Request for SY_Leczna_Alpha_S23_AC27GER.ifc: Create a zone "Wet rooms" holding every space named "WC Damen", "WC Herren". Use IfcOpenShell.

First a look at what the model holds.

```python
import ifcopenshell

model = ifcopenshell.open("SY_Leczna_Alpha_S23_AC27GER.ifc")
print(model.schema)
seen = {}
for space in model.by_type("IfcSpace"):
    seen[space.LongName] = seen.get(space.LongName, 0) + 1
for name, count in sorted(seen.items(), key=str):
    print(count, "x", name)
print("zones:", [z.Name for z in model.by_type("IfcZone")][:20])
```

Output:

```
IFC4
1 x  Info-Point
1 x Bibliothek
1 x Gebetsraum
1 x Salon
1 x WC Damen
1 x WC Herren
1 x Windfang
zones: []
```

```python
import ifcopenshell
import ifcopenshell.api.group
import ifcopenshell.api.root

model = ifcopenshell.open("SY_Leczna_Alpha_S23_AC27GER.ifc")

names = {"WC Damen", "WC Herren"}
spaces = [s for s in model.by_type("IfcSpace") if s.LongName in names]

zone = ifcopenshell.api.root.create_entity(model, ifc_class="IfcZone", name="Wet rooms")
ifcopenshell.api.group.assign_group(model, products=spaces, group=zone)
print(len(spaces), "spaces in", zone.Name)

model.write("SY_Leczna_Alpha_S23_AC27GER_rev.ifc")
```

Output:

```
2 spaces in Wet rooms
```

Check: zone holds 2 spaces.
